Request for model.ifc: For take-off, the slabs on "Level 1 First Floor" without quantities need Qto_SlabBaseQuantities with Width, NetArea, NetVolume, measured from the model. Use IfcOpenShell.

First a look at what the model holds.

```python
import ifcopenshell
import ifcopenshell.util.element
import ifcopenshell.util.unit

model = ifcopenshell.open("model.ifc")
print(model.schema)
for unit_type in ("LENGTHUNIT", "AREAUNIT", "VOLUMEUNIT"):
    print(unit_type, ifcopenshell.util.unit.calculate_unit_scale(model, unit_type))
storey = next(s for s in model.by_type("IfcBuildingStorey") if s.Name == "Level 1 First Floor")
slabs = [e for e in ifcopenshell.util.element.get_decomposition(storey) if e.is_a("IfcSlab")]
for e in sorted(slabs, key=lambda e: e.id()):
    print(e.id(), e.is_a(), e.Name, list(ifcopenshell.util.element.get_psets(e, qtos_only=True)), sep=" | ")
```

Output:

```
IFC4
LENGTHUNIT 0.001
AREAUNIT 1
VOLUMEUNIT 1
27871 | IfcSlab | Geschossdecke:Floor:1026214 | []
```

```python
import ifcopenshell
import ifcopenshell.api.pset
import ifcopenshell.geom
import ifcopenshell.util.element
import ifcopenshell.util.shape
import ifcopenshell.util.unit

model = ifcopenshell.open("model.ifc")
unit_scale = ifcopenshell.util.unit.calculate_unit_scale(model)
area_scale = ifcopenshell.util.unit.calculate_unit_scale(model, "AREAUNIT")
volume_scale = ifcopenshell.util.unit.calculate_unit_scale(model, "VOLUMEUNIT")
settings = ifcopenshell.geom.settings()

storey = next(s for s in model.by_type("IfcBuildingStorey") if s.Name == "Level 1 First Floor")
slabs = [e for e in ifcopenshell.util.element.get_decomposition(storey) if e.is_a("IfcSlab")]

for e in sorted(slabs, key=lambda e: e.id()):
    if ifcopenshell.util.element.get_psets(e, qtos_only=True, should_inherit=False):
        continue
    # Geometry comes back in metres, in the element's own axes.
    shape = ifcopenshell.geom.create_shape(settings, e)
    values = {
        "Width": ifcopenshell.util.shape.get_z(shape.geometry) / unit_scale,
        "NetArea": ifcopenshell.util.shape.get_footprint_area(shape.geometry) / area_scale,
        "NetVolume": ifcopenshell.util.shape.get_volume(shape.geometry) / volume_scale,
    }
    qto = ifcopenshell.api.pset.add_qto(model, product=e, name="Qto_SlabBaseQuantities")
    ifcopenshell.api.pset.edit_qto(model, qto=qto, properties=values)
    print(e.id(), {k: round(v, 3) for k, v in values.items()})

model.write("model_v2.ifc")
```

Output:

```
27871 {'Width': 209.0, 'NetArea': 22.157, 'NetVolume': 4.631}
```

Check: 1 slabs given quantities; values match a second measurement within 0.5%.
